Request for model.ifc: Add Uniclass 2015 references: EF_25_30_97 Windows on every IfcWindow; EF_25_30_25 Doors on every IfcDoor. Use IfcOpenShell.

First a look at what the model holds.

```python
import ifcopenshell

model = ifcopenshell.open("model.ifc")
print(model.schema)
print("classifications:", [c.Name for c in model.by_type("IfcClassification")])
for ifc_class in ("IfcDoor", "IfcRoof", "IfcStair", "IfcWall", "IfcWindow"):
    print(ifc_class, len(model.by_type(ifc_class)))
```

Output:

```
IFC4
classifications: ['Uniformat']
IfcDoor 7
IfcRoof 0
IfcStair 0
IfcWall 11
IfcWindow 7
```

```python
import ifcopenshell
import ifcopenshell.api.classification

model = ifcopenshell.open("model.ifc")

system = ifcopenshell.api.classification.add_classification(model, classification="Uniclass 2015")

codes = {
    "IfcWindow": ("EF_25_30_97", "Windows"),
    "IfcDoor": ("EF_25_30_25", "Doors"),
}
for ifc_class, (code, name) in codes.items():
    products = model.by_type(ifc_class)
    ifcopenshell.api.classification.add_reference(
        model, products=products, classification=system, identification=code, name=name
    )
    print(code, len(products))

model.write("model_v2.ifc")
```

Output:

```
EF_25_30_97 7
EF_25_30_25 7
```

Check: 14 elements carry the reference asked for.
